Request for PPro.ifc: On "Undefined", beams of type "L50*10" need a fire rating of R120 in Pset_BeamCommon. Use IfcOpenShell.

First a look at what the model holds.

```python
import ifcopenshell
import ifcopenshell.util.element

model = ifcopenshell.open("PPro.ifc")
print(model.schema)
storey = next(s for s in model.by_type("IfcBuildingStorey") if s.Name == "Undefined")
beams = [e for e in ifcopenshell.util.element.get_decomposition(storey) if e.is_a("IfcBeam")]
seen = {}
for e in beams:
    element_type = ifcopenshell.util.element.get_type(e)
    key = (element_type.Name if element_type != e and element_type else None, ifcopenshell.util.element.get_pset(e, "Pset_BeamCommon", "FireRating"))
    seen[key] = seen.get(key, 0) + 1
for (name, value), count in sorted(seen.items(), key=str):
    print(count, "x", name, "|", value)
```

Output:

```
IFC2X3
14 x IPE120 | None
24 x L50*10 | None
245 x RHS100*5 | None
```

```python
import ifcopenshell
import ifcopenshell.api.pset
import ifcopenshell.util.element

model = ifcopenshell.open("PPro.ifc")

storey = next(s for s in model.by_type("IfcBuildingStorey") if s.Name == "Undefined")
beams = [e for e in ifcopenshell.util.element.get_decomposition(storey) if e.is_a("IfcBeam")]

count = 0
for e in beams:
    element_type = ifcopenshell.util.element.get_type(e)
    if element_type in (None, e) or element_type.Name != "L50*10":
        continue
    # add_pset returns the element's existing set when there is one.
    pset = ifcopenshell.api.pset.add_pset(model, product=e, name="Pset_BeamCommon")
    ifcopenshell.api.pset.edit_pset(model, pset=pset, properties={"FireRating": "R120"})
    count += 1

print(count, "beams updated")

model.write("PPro_updated.ifc")
```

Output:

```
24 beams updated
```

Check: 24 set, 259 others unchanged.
